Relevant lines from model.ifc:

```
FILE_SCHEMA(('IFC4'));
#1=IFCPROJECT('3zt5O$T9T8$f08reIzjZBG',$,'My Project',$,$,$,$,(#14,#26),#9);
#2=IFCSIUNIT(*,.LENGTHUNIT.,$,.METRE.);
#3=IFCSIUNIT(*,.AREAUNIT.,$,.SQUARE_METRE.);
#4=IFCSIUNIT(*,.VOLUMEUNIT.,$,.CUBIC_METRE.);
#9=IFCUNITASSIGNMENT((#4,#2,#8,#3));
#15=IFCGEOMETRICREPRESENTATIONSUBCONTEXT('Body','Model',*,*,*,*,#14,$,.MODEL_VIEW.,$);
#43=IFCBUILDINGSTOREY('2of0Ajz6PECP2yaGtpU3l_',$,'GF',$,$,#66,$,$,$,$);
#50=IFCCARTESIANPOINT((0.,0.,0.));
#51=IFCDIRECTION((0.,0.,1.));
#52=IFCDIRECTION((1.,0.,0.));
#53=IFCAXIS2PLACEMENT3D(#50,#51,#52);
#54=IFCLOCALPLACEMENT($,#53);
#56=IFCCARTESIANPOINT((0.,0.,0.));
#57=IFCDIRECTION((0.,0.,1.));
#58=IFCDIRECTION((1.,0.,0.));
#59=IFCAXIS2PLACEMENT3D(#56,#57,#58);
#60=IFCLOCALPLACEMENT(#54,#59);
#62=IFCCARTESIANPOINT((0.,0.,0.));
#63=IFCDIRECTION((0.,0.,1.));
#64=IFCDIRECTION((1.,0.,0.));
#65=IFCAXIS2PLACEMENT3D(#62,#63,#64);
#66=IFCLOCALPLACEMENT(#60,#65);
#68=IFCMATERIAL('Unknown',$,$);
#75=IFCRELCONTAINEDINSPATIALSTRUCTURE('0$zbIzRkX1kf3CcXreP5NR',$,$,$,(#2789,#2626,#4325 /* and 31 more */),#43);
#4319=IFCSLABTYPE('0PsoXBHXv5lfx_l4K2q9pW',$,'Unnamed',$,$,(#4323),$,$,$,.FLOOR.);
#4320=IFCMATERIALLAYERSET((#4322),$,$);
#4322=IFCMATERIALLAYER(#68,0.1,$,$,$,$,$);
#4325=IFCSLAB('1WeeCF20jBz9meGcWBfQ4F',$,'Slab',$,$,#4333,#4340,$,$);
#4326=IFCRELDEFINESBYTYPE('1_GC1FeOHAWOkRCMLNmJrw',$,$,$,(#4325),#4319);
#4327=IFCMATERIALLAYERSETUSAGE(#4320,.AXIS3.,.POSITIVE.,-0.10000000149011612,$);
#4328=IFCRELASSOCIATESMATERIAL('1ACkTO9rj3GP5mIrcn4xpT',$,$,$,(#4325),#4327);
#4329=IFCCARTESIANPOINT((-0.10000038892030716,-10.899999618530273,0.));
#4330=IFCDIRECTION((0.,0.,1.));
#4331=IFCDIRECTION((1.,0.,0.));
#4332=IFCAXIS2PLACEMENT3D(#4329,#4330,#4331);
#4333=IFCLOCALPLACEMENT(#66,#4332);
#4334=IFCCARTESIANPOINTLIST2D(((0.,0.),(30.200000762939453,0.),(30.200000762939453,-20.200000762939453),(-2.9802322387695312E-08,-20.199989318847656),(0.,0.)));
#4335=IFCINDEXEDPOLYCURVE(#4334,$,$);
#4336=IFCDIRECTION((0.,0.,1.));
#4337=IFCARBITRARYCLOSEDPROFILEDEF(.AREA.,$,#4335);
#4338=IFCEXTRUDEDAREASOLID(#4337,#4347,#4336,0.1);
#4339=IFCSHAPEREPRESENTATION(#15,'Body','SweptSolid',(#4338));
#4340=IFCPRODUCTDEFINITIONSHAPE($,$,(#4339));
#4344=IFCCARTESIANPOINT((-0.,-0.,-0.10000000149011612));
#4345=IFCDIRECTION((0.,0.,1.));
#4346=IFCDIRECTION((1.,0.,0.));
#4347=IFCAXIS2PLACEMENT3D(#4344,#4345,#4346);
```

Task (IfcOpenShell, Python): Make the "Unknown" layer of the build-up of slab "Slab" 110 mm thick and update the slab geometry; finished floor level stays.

```python
import ifcopenshell
import ifcopenshell.util.element
import ifcopenshell.util.representation
import ifcopenshell.util.unit

model = ifcopenshell.open("model.ifc")
unit_scale = ifcopenshell.util.unit.calculate_unit_scale(model)

layer_set = model.by_id(4320)
layer = next(l for l in layer_set.MaterialLayers if l.Material and l.Material.Name == "Unknown")
change = 0.11 / unit_scale - layer.LayerThickness
layer.LayerThickness += change

# Geometry does not follow the layer set by itself.
slabs = [e for e in ifcopenshell.util.element.get_elements_by_material(model, layer_set) if e.is_a("IfcSlab")]
for slab in sorted(slabs, key=lambda e: e.id()):
    body = ifcopenshell.util.representation.get_representation(slab, "Model", "Body")
    solid = body.Items[0]
    old_depth = solid.Depth
    solid.Depth += change
    # Extruded upwards: lower the start of the extrusion so the top stays.
    x, y, z = solid.Position.Location.Coordinates
    solid.Position.Location = model.createIfcCartesianPoint((x, y, z - change))
    print(slab.id(), f"{old_depth:g} -> {solid.Depth:g}")

# The layers are counted up from the underside, which has moved.
for usage in {ifcopenshell.util.element.get_material(slab) for slab in slabs}:
    usage.OffsetFromReferenceLine -= change

model.write("model_v2.ifc")
```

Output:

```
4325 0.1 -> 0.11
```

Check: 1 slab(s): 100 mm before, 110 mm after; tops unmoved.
